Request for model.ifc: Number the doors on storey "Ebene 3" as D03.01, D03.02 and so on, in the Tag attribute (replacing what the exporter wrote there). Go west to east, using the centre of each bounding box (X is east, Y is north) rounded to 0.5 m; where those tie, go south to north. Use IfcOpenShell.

First a look at what the model holds.

```python
import ifcopenshell
import ifcopenshell.util.element
import ifcopenshell.util.placement

model = ifcopenshell.open("model.ifc")
print(model.schema)
storey = next(s for s in model.by_type("IfcBuildingStorey") if s.Name == "Ebene 3")
doors = [e for e in ifcopenshell.util.element.get_decomposition(storey) if e.is_a("IfcDoor")]
for e in sorted(doors, key=lambda e: e.id()):
    origin = ifcopenshell.util.placement.get_local_placement(e.ObjectPlacement)[:3, 3]
    print(e.id(), e.Tag, e.Name, origin.round(2) + 0.0, sep=" | ")
```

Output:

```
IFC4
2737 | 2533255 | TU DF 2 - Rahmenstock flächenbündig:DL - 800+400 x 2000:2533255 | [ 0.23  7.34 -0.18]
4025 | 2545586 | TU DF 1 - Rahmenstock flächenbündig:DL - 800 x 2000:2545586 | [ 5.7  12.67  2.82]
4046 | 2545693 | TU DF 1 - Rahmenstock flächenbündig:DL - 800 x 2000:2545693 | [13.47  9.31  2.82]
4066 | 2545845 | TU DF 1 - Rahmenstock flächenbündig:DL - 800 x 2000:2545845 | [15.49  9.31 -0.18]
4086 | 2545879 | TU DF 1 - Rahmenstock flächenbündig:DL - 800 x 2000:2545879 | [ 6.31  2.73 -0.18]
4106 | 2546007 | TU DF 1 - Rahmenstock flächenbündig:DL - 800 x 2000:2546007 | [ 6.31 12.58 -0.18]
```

```python
import ifcopenshell
import ifcopenshell.geom
import ifcopenshell.util.element
import ifcopenshell.util.shape

model = ifcopenshell.open("model.ifc")
settings = ifcopenshell.geom.settings()
settings.set("use-world-coords", True)


def centre(element):
    shape = ifcopenshell.geom.create_shape(settings, element)
    return ifcopenshell.util.shape.get_bbox_centroid(shape.geometry)


storey = next(s for s in model.by_type("IfcBuildingStorey") if s.Name == "Ebene 3")
doors = [e for e in ifcopenshell.util.element.get_decomposition(storey) if e.is_a("IfcDoor")]

# Insertion points can sit at a corner or the storey origin, so sort by the geometry (in metres).
centres = {e: centre(e) for e in doors}
doors.sort(key=lambda e: (round(centres[e][0] / 0.5), centres[e][1]))

for i, e in enumerate(doors, start=1):
    number = f"D03.{i:02d}"
    e.Tag = number
    print(e.id(), number)

model.write("model_updated.ifc")
```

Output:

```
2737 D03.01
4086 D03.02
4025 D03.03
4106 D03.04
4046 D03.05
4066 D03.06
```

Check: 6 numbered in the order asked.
